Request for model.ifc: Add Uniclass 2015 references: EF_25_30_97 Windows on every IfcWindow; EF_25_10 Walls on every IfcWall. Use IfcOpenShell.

First a look at what the model holds.

```python
import ifcopenshell

model = ifcopenshell.open("model.ifc")
print(model.schema)
print("classifications:", [c.Name for c in model.by_type("IfcClassification")])
for ifc_class in ("IfcDoor", "IfcRoof", "IfcStair", "IfcWall", "IfcWindow"):
    print(ifc_class, len(model.by_type(ifc_class)))
```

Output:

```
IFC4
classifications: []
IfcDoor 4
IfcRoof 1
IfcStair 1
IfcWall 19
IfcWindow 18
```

```python
import ifcopenshell
import ifcopenshell.api.classification

model = ifcopenshell.open("model.ifc")

system = ifcopenshell.api.classification.add_classification(model, classification="Uniclass 2015")

codes = {
    "IfcWindow": ("EF_25_30_97", "Windows"),
    "IfcWall": ("EF_25_10", "Walls"),
}
for ifc_class, (code, name) in codes.items():
    products = model.by_type(ifc_class)
    ifcopenshell.api.classification.add_reference(
        model, products=products, classification=system, identification=code, name=name
    )
    print(code, len(products))

model.write("model-out.ifc")
```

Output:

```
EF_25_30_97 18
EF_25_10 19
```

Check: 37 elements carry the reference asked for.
